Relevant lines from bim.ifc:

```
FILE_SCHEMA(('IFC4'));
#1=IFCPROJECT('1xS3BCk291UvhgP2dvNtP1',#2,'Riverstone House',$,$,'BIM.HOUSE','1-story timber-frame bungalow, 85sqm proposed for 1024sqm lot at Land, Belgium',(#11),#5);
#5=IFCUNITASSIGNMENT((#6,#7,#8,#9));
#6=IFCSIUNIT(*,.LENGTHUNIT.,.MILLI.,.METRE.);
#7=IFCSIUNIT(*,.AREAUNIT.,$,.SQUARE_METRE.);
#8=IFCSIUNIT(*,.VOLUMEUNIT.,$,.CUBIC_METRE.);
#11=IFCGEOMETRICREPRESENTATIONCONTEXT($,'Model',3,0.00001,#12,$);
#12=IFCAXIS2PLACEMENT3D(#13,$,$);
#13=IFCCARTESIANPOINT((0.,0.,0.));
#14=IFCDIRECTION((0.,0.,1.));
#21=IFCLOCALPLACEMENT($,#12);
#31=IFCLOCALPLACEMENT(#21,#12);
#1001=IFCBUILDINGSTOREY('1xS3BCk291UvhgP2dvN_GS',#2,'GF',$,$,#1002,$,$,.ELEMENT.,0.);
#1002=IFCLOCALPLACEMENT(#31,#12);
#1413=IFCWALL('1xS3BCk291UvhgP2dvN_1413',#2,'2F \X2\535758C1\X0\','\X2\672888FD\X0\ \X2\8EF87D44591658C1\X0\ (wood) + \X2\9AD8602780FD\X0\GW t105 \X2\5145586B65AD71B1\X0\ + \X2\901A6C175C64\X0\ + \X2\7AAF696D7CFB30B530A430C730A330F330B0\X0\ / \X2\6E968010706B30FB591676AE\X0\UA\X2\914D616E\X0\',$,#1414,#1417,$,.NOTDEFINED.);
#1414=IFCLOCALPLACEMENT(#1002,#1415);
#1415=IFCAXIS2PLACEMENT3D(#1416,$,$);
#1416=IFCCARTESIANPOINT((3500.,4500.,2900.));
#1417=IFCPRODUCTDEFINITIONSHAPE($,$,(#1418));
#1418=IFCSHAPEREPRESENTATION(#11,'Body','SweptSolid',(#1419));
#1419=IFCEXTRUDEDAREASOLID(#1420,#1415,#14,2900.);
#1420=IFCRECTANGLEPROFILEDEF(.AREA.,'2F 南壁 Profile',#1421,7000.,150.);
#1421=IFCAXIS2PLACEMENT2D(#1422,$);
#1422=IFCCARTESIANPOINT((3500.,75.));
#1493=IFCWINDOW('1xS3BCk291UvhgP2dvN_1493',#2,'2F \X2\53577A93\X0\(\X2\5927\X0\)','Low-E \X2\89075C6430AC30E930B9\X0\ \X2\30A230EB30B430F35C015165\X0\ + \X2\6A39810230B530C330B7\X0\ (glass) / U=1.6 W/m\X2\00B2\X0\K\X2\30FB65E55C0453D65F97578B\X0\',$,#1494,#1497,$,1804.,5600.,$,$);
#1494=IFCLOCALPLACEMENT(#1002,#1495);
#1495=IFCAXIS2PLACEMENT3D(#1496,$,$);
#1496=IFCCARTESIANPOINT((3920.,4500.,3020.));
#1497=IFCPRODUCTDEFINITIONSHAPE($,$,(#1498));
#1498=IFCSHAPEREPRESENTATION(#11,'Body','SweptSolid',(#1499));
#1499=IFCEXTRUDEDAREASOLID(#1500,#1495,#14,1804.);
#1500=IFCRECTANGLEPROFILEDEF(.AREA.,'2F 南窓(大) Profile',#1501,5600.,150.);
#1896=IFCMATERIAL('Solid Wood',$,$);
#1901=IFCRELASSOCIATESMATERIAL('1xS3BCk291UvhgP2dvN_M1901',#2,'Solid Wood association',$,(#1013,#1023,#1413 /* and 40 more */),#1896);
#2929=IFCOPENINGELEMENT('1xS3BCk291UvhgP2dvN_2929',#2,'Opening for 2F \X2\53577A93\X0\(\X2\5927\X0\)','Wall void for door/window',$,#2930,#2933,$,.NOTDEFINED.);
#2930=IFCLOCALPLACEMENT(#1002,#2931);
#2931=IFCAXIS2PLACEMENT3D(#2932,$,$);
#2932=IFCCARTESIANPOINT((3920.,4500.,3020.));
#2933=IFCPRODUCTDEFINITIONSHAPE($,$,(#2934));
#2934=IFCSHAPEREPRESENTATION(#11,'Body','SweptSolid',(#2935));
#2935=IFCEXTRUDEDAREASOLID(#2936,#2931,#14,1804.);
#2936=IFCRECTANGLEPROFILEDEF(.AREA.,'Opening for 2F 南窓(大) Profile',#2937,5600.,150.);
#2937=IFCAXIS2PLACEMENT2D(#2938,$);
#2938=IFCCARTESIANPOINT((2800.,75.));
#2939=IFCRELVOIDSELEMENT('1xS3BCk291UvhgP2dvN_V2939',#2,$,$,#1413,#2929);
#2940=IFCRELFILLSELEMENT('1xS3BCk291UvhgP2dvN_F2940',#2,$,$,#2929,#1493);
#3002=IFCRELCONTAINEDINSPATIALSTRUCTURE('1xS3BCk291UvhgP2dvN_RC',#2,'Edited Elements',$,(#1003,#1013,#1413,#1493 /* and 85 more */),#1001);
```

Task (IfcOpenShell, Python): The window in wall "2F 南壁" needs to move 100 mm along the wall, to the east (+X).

```python
import ifcopenshell
import ifcopenshell.api.geometry
import ifcopenshell.util.placement
import ifcopenshell.util.unit

model = ifcopenshell.open("bim.ifc")
unit_scale = ifcopenshell.util.unit.calculate_unit_scale(model)

window = model.by_id(1493)
opening = window.FillsVoids[0].RelatingOpeningElement
wall = opening.VoidsElements[0].RelatingBuildingElement

wall_matrix = ifcopenshell.util.placement.get_local_placement(wall.ObjectPlacement)
shift = wall_matrix[:3, 0] * 0.1 / unit_scale
before = ifcopenshell.util.placement.get_local_placement(window.ObjectPlacement)[:3, 3].copy()

# The window is not placed relative to its opening, so move both.
for product in (opening, window):
    matrix = ifcopenshell.util.placement.get_local_placement(product.ObjectPlacement)
    matrix[:3, 3] += shift
    ifcopenshell.api.geometry.edit_object_placement(model, product=product, matrix=matrix, is_si=False)

after = ifcopenshell.util.placement.get_local_placement(window.ObjectPlacement)[:3, 3]
print("window moved by", (after - before).round(3) + 0.0)

model.write("bim_rev.ifc")
```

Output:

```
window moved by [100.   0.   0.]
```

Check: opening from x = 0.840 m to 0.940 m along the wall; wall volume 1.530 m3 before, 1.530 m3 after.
